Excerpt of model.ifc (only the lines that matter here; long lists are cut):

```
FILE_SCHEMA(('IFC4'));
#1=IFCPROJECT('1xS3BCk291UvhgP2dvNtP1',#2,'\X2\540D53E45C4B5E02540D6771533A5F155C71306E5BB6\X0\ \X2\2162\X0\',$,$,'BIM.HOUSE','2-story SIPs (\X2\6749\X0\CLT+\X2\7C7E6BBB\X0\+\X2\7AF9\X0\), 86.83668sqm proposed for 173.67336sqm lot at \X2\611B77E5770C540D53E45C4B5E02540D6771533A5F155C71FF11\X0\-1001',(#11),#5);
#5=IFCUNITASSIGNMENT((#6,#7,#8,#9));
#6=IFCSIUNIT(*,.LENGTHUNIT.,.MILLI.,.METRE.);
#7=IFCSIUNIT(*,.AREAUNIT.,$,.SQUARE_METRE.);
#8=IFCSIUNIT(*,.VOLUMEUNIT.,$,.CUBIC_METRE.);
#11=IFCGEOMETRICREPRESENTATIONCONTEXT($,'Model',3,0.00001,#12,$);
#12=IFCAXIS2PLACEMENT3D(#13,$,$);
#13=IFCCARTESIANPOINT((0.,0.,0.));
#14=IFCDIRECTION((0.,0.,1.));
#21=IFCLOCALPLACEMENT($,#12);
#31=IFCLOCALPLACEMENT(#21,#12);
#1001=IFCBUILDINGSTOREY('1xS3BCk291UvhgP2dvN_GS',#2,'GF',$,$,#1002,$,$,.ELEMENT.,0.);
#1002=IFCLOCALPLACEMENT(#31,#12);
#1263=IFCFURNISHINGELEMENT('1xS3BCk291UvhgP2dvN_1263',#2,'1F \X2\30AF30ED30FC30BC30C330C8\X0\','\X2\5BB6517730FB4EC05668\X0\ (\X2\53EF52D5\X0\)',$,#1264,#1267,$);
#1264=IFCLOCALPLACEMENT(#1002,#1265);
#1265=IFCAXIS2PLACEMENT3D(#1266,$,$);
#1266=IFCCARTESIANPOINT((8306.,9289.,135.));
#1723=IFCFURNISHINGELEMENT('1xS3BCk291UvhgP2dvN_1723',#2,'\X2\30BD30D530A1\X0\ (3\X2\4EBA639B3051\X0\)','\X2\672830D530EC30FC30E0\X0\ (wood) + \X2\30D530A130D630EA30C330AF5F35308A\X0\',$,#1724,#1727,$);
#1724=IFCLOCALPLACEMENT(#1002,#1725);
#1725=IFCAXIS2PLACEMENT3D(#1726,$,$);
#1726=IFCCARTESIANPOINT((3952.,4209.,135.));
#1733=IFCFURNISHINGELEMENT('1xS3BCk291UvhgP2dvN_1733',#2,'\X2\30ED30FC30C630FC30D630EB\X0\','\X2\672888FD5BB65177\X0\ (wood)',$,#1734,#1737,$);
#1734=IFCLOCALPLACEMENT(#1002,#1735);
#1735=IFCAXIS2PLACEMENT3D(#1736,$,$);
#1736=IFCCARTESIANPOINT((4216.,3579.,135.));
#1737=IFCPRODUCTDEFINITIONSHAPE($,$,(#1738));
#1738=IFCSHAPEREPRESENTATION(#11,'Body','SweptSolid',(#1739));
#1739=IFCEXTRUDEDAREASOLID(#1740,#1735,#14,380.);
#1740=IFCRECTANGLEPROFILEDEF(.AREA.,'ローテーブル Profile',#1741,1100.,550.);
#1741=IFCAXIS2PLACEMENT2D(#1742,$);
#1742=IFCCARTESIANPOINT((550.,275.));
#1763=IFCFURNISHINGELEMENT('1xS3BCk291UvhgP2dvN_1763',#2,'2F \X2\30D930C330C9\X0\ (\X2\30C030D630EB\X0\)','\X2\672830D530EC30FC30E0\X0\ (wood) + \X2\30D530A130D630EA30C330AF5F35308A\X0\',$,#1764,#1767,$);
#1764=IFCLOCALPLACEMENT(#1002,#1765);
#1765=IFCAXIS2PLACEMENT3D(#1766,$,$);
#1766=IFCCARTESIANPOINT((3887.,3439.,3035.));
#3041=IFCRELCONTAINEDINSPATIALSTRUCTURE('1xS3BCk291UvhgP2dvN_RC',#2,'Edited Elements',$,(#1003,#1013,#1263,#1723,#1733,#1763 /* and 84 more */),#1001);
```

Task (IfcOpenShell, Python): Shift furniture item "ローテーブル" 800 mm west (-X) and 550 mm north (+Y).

```python
import ifcopenshell
import ifcopenshell.api.geometry
import ifcopenshell.util.placement
import ifcopenshell.util.unit

model = ifcopenshell.open("model.ifc")
unit_scale = ifcopenshell.util.unit.calculate_unit_scale(model)

item = model.by_guid("1xS3BCk291UvhgP2dvN_1733")
matrix = ifcopenshell.util.placement.get_local_placement(item.ObjectPlacement)
matrix[0, 3] -= 0.8 / unit_scale
matrix[1, 3] += 0.55 / unit_scale
ifcopenshell.api.geometry.edit_object_placement(model, product=item, matrix=matrix, is_si=False)

print(ifcopenshell.util.placement.get_local_placement(item.ObjectPlacement).round(3) + 0.0)

model.write("model-out.ifc")
```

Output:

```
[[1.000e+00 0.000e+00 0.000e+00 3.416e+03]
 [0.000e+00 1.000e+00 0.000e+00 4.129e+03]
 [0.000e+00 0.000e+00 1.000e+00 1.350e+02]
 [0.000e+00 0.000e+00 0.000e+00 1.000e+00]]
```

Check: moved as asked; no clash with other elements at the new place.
